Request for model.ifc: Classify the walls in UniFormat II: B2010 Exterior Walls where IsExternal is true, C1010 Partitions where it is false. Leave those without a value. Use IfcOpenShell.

First a look at what the model holds.

```python
import ifcopenshell
import ifcopenshell.util.element

model = ifcopenshell.open("model.ifc")
print(model.schema)
print("classifications:", [c.Name for c in model.by_type("IfcClassification")])
values = [ifcopenshell.util.element.get_pset(e, "Pset_WallCommon", "IsExternal") for e in model.by_type("IfcWall")]
for value in (True, False, None):
    print("IsExternal", value, values.count(value))
```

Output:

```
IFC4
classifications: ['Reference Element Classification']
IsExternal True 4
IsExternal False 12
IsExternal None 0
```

```python
import ifcopenshell
import ifcopenshell.api.classification
import ifcopenshell.util.element

model = ifcopenshell.open("model.ifc")

system = ifcopenshell.api.classification.add_classification(model, classification="UniFormat II")

walls = model.by_type("IfcWall")
external = {e: ifcopenshell.util.element.get_pset(e, "Pset_WallCommon", "IsExternal") for e in walls}
for flag, code, name in ((True, "B2010", "Exterior Walls"), (False, "C1010", "Partitions")):
    products = [e for e in walls if external[e] is flag]
    ifcopenshell.api.classification.add_reference(
        model, products=products, classification=system, identification=code, name=name
    )
    print(code, len(products))

model.write("model_rev.ifc")
```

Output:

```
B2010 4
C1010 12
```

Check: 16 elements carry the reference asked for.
